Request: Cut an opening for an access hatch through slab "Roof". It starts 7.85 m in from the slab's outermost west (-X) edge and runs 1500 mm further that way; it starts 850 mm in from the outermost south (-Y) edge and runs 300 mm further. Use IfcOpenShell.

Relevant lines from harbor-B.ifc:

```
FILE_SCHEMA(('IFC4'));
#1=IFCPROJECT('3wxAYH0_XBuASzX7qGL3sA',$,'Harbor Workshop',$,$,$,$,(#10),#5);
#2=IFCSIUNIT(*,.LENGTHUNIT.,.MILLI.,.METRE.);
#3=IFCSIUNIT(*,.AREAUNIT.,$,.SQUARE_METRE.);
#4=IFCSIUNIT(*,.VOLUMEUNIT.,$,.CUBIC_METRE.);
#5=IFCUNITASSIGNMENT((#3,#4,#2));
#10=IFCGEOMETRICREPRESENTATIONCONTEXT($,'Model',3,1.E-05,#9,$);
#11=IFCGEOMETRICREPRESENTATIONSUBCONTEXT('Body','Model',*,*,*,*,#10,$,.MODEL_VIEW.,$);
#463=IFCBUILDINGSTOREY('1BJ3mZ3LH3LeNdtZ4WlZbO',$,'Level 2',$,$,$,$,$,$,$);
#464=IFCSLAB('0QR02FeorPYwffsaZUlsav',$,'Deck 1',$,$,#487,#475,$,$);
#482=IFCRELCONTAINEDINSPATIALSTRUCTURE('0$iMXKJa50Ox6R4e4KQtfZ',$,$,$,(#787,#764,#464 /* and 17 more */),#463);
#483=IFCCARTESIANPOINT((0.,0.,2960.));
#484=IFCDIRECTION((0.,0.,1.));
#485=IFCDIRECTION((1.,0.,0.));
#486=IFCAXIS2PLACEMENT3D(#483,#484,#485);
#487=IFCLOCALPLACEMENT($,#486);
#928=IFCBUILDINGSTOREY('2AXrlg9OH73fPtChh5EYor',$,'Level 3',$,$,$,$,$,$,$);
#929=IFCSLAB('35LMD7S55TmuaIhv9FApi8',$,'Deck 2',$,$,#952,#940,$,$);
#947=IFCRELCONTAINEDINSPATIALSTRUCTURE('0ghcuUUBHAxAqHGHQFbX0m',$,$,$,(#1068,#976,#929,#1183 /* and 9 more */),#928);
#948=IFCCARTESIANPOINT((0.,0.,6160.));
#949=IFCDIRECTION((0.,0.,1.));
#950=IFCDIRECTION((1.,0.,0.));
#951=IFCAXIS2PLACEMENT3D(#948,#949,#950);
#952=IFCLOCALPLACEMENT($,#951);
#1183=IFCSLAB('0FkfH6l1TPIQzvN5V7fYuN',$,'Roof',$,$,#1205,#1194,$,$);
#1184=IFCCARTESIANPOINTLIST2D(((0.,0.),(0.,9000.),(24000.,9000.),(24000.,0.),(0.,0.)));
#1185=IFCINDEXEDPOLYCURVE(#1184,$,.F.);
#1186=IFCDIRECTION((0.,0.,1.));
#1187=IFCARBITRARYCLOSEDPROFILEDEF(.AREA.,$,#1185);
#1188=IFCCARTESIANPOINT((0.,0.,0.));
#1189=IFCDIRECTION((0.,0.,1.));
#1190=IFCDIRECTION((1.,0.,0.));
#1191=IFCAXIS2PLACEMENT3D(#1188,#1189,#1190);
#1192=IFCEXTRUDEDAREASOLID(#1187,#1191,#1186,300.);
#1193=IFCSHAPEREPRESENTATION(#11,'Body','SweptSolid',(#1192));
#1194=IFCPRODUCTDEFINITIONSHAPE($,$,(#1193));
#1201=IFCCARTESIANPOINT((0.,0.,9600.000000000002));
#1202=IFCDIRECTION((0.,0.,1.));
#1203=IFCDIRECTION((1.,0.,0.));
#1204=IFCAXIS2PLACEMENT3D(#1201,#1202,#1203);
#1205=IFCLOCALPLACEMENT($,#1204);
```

```python
import numpy as np
import ifcopenshell
import ifcopenshell.api.feature
import ifcopenshell.api.geometry
import ifcopenshell.api.root
import ifcopenshell.geom
import ifcopenshell.util.placement
import ifcopenshell.util.representation
import ifcopenshell.util.shape
import ifcopenshell.util.unit

model = ifcopenshell.open("harbor-B.ifc")
unit_scale = ifcopenshell.util.unit.calculate_unit_scale(model)
settings = ifcopenshell.geom.settings()


def volume(element):
    """Net volume in cubic metres, openings subtracted."""
    shape = ifcopenshell.geom.create_shape(settings, element)
    return ifcopenshell.util.shape.get_volume(shape.geometry)


slab = model.by_guid("0FkfH6l1TPIQzvN5V7fYuN")
before = volume(slab)

# Extent in the slab's own axes, in metres. The edges named are its -X and -Y sides.
slab_shape = ifcopenshell.geom.create_shape(settings, slab)
vertices = ifcopenshell.util.shape.get_vertices(slab_shape.geometry)
x_min, y_min, bottom = vertices.min(axis=0)
top = vertices[:, 2].max()

opening = ifcopenshell.api.root.create_entity(model, ifc_class="IfcOpeningElement", name="Access hatch opening", predefined_type="OPENING")
context = ifcopenshell.util.representation.get_context(model, "Model", "Body", "MODEL_VIEW")
width, depth = 1.5, 0.3
outline = [(0.0, 0.0), (width, 0.0), (width, depth), (0.0, depth), (0.0, 0.0)]
# Overshoot both faces by 50 mm so the cut is clean.
shape = ifcopenshell.api.geometry.add_slab_representation(
    model, context=context, depth=top - bottom + 0.1, polyline=outline
)
ifcopenshell.api.geometry.assign_representation(model, product=opening, representation=shape)

matrix = ifcopenshell.util.placement.get_local_placement(slab.ObjectPlacement)
matrix[:, 3] = matrix @ np.append(np.array([x_min + 7.85, y_min + 0.85, bottom - 0.05]) / unit_scale, 1.0)
ifcopenshell.api.geometry.edit_object_placement(model, product=opening, matrix=matrix, is_si=False)
ifcopenshell.api.feature.add_feature(model, feature=opening, element=slab)

after = volume(slab)

print(f"slab volume {before:.3f} -> {after:.3f} m3")

model.write("harbor-B_edited.ifc")
```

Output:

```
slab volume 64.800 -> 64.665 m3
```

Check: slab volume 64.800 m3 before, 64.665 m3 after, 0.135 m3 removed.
